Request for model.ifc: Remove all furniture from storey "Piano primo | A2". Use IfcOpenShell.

First a look at what the model holds.

```python
import ifcopenshell
import ifcopenshell.util.element

model = ifcopenshell.open("model.ifc")
print(model.schema)
storey = next(s for s in model.by_type("IfcBuildingStorey") if s.Name == "Piano primo | A2")
furniture = [e for e in ifcopenshell.util.element.get_decomposition(storey) if e.is_a("IfcFurnishingElement")]
seen = {}
for e in furniture:
    element_type = ifcopenshell.util.element.get_type(e)
    name = element_type.Name if element_type not in (None, e) else None
    seen[name] = seen.get(name, 0) + 1
for name, count in sorted(seen.items(), key=str):
    print(count, "x", name)
```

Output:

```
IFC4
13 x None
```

```python
import ifcopenshell
import ifcopenshell.api.root
import ifcopenshell.util.element

model = ifcopenshell.open("model.ifc")

storey = next(s for s in model.by_type("IfcBuildingStorey") if s.Name == "Piano primo | A2")
furniture = [e for e in ifcopenshell.util.element.get_decomposition(storey) if e.is_a("IfcFurnishingElement")]

for e in furniture:
    ifcopenshell.api.root.remove_product(model, product=e)
print(len(furniture), "removed")

model.write("model_updated.ifc")
```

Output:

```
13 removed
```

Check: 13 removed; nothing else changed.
